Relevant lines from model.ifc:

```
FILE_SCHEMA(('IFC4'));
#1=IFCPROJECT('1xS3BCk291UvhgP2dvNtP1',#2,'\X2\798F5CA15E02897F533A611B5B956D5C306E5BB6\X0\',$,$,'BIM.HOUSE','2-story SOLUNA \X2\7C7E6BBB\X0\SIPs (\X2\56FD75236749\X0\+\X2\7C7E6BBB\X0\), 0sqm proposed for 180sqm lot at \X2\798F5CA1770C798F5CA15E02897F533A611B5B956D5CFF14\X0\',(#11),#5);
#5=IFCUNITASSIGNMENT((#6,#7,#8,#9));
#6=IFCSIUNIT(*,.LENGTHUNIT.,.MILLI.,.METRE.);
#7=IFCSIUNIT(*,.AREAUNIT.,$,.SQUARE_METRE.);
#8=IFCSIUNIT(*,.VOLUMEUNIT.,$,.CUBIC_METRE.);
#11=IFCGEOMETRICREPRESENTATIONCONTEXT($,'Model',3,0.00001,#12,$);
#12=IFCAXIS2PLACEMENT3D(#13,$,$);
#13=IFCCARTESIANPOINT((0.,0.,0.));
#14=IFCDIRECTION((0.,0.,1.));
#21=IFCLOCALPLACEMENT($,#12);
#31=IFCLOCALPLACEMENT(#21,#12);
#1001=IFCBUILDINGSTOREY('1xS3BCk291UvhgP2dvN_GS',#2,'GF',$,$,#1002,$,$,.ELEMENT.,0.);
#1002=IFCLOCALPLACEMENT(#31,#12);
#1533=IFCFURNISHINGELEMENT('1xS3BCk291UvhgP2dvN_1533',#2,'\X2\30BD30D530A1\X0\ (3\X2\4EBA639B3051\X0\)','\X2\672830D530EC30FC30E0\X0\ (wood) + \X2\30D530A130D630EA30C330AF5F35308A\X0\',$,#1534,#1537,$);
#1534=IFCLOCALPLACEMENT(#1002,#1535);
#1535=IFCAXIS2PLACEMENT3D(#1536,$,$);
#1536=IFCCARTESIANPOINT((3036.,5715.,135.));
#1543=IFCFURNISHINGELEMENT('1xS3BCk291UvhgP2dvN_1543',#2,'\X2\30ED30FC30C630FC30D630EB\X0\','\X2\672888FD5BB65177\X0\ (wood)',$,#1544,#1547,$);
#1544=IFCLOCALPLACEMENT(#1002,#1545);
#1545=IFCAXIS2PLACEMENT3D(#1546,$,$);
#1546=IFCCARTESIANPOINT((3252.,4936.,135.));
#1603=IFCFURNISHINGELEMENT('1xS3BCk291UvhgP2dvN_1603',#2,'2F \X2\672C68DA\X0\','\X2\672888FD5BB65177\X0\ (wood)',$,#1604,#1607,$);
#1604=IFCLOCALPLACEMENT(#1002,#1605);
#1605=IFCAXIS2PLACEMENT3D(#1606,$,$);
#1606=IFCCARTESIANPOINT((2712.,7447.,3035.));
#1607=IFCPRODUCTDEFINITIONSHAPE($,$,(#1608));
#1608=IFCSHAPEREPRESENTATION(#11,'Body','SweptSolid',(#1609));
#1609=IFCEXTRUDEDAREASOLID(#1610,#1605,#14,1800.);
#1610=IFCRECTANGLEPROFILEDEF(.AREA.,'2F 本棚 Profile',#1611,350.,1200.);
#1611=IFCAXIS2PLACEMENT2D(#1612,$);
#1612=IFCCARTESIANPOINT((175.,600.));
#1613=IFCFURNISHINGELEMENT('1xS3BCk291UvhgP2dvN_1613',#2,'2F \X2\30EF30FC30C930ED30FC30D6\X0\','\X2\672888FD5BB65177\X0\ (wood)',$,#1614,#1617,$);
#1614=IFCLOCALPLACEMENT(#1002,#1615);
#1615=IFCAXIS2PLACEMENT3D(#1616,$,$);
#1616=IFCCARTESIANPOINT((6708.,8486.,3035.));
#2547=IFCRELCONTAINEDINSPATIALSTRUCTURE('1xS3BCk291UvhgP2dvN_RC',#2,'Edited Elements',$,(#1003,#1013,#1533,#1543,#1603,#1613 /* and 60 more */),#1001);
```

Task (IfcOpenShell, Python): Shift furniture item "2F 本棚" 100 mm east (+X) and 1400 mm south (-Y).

```python
import ifcopenshell
import ifcopenshell.api.geometry
import ifcopenshell.util.placement
import ifcopenshell.util.unit

model = ifcopenshell.open("model.ifc")
unit_scale = ifcopenshell.util.unit.calculate_unit_scale(model)

item = model.by_guid("1xS3BCk291UvhgP2dvN_1603")
matrix = ifcopenshell.util.placement.get_local_placement(item.ObjectPlacement)
matrix[0, 3] += 0.1 / unit_scale
matrix[1, 3] -= 1.4 / unit_scale
ifcopenshell.api.geometry.edit_object_placement(model, product=item, matrix=matrix, is_si=False)

print(ifcopenshell.util.placement.get_local_placement(item.ObjectPlacement).round(3) + 0.0)

model.write("model_edited.ifc")
```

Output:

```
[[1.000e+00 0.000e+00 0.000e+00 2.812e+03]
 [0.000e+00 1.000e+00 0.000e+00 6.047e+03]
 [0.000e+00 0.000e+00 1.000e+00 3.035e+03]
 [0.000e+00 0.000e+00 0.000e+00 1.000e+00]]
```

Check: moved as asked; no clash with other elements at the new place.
